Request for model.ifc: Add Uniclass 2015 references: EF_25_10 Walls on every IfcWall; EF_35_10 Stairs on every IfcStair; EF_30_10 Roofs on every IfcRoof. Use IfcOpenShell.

First a look at what the model holds.

```python
import ifcopenshell

model = ifcopenshell.open("model.ifc")
print(model.schema)
print("classifications:", [c.Name for c in model.by_type("IfcClassification")])
for ifc_class in ("IfcDoor", "IfcRoof", "IfcStair", "IfcWall", "IfcWindow"):
    print(ifc_class, len(model.by_type(ifc_class)))
```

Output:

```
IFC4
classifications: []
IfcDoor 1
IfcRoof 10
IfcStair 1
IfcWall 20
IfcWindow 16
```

```python
import ifcopenshell
import ifcopenshell.api.classification

model = ifcopenshell.open("model.ifc")

system = ifcopenshell.api.classification.add_classification(model, classification="Uniclass 2015")

codes = {
    "IfcWall": ("EF_25_10", "Walls"),
    "IfcStair": ("EF_35_10", "Stairs"),
    "IfcRoof": ("EF_30_10", "Roofs"),
}
for ifc_class, (code, name) in codes.items():
    products = model.by_type(ifc_class)
    ifcopenshell.api.classification.add_reference(
        model, products=products, classification=system, identification=code, name=name
    )
    print(code, len(products))

model.write("model_edited.ifc")
```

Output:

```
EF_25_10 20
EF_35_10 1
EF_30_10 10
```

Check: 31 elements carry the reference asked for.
